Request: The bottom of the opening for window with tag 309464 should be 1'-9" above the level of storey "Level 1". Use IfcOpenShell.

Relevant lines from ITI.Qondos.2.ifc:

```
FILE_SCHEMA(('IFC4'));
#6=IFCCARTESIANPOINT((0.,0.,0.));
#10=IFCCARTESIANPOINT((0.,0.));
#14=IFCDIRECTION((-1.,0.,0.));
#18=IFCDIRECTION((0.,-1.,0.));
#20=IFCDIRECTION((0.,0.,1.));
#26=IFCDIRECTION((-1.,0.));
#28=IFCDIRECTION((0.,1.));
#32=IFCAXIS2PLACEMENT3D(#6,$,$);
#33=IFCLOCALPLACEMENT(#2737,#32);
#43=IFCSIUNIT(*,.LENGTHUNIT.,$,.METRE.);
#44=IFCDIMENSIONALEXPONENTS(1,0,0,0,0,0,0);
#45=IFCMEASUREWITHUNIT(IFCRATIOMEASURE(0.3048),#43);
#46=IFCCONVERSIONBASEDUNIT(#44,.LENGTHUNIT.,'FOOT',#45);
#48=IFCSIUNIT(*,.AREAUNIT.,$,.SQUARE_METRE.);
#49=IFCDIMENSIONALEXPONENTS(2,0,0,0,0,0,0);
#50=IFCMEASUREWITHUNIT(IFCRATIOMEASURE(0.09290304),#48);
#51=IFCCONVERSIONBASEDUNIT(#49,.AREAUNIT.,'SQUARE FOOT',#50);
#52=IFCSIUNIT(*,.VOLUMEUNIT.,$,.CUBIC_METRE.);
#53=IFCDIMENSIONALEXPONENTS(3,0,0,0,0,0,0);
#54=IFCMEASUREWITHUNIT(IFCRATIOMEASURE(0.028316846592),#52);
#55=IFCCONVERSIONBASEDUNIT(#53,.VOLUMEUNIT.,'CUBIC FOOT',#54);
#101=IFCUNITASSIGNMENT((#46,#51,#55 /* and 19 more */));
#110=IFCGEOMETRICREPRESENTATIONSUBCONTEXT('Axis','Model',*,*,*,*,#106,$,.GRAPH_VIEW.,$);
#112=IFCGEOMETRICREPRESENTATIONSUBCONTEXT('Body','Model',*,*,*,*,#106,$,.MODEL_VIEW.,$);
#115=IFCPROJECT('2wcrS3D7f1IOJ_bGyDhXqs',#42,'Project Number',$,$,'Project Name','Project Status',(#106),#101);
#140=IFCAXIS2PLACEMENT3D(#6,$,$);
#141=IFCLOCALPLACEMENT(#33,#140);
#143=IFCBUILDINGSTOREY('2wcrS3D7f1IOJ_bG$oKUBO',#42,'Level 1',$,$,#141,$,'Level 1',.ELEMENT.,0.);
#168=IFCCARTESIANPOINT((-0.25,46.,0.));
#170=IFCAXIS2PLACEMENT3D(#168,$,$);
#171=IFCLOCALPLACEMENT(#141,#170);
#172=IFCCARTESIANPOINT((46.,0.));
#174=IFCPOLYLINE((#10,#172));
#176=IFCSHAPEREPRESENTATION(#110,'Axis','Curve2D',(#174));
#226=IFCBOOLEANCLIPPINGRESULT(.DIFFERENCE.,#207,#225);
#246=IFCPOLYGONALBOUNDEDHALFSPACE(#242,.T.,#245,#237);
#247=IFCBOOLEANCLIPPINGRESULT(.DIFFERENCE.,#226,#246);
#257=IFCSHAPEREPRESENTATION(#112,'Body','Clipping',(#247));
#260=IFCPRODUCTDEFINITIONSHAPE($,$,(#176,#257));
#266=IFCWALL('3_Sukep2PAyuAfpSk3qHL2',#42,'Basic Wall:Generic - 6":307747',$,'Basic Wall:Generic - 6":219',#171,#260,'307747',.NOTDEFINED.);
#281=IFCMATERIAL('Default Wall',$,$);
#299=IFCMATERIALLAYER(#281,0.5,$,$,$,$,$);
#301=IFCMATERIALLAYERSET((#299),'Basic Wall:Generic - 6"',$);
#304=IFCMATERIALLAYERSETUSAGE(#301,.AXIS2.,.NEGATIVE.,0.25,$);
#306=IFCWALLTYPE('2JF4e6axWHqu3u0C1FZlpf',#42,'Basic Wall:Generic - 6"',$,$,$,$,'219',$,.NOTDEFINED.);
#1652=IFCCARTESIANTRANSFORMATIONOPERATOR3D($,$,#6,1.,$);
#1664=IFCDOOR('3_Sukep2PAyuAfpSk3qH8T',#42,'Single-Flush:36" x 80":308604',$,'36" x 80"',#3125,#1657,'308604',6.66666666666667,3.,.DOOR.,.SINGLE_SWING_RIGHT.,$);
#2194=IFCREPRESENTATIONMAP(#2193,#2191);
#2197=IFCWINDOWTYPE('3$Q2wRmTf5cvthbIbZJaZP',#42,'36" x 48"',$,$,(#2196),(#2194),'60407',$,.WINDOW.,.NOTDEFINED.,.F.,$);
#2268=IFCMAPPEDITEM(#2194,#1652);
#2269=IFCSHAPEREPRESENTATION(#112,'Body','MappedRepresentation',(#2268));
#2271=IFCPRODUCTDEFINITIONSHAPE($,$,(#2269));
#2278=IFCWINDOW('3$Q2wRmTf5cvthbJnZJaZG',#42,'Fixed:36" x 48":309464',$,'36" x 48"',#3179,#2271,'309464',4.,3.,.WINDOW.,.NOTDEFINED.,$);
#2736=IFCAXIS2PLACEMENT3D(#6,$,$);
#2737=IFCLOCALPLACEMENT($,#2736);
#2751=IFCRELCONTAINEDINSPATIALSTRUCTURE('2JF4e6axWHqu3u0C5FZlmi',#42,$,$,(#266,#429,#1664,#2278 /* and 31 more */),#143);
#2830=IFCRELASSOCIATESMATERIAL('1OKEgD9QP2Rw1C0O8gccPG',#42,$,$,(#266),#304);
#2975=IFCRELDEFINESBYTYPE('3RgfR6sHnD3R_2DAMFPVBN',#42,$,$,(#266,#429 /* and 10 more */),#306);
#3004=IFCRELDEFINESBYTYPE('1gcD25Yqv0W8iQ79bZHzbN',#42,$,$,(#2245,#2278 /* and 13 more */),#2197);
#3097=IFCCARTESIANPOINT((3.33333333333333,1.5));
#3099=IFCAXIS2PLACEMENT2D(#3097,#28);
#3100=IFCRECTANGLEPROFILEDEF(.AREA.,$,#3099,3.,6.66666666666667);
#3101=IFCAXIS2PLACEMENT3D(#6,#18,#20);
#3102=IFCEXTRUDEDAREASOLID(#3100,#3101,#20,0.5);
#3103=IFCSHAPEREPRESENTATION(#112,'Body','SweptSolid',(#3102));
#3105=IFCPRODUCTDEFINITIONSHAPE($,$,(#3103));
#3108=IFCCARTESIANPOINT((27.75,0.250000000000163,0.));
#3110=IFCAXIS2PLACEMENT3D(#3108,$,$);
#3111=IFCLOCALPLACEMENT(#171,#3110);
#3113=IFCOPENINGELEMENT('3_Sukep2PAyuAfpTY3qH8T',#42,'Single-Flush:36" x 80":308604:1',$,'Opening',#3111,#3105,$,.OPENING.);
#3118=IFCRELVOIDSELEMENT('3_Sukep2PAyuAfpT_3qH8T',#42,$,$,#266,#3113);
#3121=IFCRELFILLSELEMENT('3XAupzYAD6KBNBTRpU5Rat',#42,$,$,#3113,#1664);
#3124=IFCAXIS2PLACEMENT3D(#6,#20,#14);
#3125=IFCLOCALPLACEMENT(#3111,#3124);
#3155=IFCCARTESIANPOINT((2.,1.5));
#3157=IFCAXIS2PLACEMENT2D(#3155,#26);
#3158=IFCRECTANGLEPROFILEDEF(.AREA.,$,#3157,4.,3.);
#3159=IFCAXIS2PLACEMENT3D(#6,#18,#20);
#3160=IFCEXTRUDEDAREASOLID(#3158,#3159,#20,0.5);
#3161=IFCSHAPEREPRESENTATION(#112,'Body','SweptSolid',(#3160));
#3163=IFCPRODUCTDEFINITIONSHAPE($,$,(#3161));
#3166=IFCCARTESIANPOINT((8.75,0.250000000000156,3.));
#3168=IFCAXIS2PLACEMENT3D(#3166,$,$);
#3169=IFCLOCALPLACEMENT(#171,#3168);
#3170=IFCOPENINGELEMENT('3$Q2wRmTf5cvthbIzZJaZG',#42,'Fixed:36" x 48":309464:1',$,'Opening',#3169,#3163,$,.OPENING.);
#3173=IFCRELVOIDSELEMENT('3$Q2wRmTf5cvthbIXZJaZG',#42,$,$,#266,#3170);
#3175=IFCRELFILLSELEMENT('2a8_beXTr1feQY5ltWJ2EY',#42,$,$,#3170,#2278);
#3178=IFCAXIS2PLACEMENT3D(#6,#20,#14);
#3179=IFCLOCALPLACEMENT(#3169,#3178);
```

```python
import numpy as np
import ifcopenshell
import ifcopenshell.api.geometry
import ifcopenshell.geom
import ifcopenshell.util.element
import ifcopenshell.util.placement
import ifcopenshell.util.shape
import ifcopenshell.util.unit

model = ifcopenshell.open("ITI.Qondos.2.ifc")
unit_scale = ifcopenshell.util.unit.calculate_unit_scale(model)

window = model.by_id(2278)
opening = window.FillsVoids[0].RelatingOpeningElement
storey = ifcopenshell.util.element.get_container(window, ifc_class="IfcBuildingStorey")
level = ifcopenshell.util.placement.get_local_placement(storey.ObjectPlacement)[2, 3]

# The opening's origin need not be at the sill, so measure its lowest point.
shape = ifcopenshell.geom.create_shape(ifcopenshell.geom.settings(), opening)
bottom = ifcopenshell.util.shape.get_shape_bottom_elevation(shape, shape.geometry) / unit_scale
dz = level + 21 * 0.0254 / unit_scale - bottom

shift = np.array([0.0, 0.0, dz])
# The window is placed relative to its opening, so it follows when the opening moves.
matrix = ifcopenshell.util.placement.get_local_placement(opening.ObjectPlacement)
matrix[:3, 3] += shift
ifcopenshell.api.geometry.edit_object_placement(
    model, product=opening, matrix=matrix, is_si=False, should_transform_children=True
)

print(f"moved by {dz * unit_scale:+.3f} m")

model.write("ITI.Qondos.2-out.ifc")
```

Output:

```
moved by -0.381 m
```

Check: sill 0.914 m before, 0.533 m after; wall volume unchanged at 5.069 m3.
